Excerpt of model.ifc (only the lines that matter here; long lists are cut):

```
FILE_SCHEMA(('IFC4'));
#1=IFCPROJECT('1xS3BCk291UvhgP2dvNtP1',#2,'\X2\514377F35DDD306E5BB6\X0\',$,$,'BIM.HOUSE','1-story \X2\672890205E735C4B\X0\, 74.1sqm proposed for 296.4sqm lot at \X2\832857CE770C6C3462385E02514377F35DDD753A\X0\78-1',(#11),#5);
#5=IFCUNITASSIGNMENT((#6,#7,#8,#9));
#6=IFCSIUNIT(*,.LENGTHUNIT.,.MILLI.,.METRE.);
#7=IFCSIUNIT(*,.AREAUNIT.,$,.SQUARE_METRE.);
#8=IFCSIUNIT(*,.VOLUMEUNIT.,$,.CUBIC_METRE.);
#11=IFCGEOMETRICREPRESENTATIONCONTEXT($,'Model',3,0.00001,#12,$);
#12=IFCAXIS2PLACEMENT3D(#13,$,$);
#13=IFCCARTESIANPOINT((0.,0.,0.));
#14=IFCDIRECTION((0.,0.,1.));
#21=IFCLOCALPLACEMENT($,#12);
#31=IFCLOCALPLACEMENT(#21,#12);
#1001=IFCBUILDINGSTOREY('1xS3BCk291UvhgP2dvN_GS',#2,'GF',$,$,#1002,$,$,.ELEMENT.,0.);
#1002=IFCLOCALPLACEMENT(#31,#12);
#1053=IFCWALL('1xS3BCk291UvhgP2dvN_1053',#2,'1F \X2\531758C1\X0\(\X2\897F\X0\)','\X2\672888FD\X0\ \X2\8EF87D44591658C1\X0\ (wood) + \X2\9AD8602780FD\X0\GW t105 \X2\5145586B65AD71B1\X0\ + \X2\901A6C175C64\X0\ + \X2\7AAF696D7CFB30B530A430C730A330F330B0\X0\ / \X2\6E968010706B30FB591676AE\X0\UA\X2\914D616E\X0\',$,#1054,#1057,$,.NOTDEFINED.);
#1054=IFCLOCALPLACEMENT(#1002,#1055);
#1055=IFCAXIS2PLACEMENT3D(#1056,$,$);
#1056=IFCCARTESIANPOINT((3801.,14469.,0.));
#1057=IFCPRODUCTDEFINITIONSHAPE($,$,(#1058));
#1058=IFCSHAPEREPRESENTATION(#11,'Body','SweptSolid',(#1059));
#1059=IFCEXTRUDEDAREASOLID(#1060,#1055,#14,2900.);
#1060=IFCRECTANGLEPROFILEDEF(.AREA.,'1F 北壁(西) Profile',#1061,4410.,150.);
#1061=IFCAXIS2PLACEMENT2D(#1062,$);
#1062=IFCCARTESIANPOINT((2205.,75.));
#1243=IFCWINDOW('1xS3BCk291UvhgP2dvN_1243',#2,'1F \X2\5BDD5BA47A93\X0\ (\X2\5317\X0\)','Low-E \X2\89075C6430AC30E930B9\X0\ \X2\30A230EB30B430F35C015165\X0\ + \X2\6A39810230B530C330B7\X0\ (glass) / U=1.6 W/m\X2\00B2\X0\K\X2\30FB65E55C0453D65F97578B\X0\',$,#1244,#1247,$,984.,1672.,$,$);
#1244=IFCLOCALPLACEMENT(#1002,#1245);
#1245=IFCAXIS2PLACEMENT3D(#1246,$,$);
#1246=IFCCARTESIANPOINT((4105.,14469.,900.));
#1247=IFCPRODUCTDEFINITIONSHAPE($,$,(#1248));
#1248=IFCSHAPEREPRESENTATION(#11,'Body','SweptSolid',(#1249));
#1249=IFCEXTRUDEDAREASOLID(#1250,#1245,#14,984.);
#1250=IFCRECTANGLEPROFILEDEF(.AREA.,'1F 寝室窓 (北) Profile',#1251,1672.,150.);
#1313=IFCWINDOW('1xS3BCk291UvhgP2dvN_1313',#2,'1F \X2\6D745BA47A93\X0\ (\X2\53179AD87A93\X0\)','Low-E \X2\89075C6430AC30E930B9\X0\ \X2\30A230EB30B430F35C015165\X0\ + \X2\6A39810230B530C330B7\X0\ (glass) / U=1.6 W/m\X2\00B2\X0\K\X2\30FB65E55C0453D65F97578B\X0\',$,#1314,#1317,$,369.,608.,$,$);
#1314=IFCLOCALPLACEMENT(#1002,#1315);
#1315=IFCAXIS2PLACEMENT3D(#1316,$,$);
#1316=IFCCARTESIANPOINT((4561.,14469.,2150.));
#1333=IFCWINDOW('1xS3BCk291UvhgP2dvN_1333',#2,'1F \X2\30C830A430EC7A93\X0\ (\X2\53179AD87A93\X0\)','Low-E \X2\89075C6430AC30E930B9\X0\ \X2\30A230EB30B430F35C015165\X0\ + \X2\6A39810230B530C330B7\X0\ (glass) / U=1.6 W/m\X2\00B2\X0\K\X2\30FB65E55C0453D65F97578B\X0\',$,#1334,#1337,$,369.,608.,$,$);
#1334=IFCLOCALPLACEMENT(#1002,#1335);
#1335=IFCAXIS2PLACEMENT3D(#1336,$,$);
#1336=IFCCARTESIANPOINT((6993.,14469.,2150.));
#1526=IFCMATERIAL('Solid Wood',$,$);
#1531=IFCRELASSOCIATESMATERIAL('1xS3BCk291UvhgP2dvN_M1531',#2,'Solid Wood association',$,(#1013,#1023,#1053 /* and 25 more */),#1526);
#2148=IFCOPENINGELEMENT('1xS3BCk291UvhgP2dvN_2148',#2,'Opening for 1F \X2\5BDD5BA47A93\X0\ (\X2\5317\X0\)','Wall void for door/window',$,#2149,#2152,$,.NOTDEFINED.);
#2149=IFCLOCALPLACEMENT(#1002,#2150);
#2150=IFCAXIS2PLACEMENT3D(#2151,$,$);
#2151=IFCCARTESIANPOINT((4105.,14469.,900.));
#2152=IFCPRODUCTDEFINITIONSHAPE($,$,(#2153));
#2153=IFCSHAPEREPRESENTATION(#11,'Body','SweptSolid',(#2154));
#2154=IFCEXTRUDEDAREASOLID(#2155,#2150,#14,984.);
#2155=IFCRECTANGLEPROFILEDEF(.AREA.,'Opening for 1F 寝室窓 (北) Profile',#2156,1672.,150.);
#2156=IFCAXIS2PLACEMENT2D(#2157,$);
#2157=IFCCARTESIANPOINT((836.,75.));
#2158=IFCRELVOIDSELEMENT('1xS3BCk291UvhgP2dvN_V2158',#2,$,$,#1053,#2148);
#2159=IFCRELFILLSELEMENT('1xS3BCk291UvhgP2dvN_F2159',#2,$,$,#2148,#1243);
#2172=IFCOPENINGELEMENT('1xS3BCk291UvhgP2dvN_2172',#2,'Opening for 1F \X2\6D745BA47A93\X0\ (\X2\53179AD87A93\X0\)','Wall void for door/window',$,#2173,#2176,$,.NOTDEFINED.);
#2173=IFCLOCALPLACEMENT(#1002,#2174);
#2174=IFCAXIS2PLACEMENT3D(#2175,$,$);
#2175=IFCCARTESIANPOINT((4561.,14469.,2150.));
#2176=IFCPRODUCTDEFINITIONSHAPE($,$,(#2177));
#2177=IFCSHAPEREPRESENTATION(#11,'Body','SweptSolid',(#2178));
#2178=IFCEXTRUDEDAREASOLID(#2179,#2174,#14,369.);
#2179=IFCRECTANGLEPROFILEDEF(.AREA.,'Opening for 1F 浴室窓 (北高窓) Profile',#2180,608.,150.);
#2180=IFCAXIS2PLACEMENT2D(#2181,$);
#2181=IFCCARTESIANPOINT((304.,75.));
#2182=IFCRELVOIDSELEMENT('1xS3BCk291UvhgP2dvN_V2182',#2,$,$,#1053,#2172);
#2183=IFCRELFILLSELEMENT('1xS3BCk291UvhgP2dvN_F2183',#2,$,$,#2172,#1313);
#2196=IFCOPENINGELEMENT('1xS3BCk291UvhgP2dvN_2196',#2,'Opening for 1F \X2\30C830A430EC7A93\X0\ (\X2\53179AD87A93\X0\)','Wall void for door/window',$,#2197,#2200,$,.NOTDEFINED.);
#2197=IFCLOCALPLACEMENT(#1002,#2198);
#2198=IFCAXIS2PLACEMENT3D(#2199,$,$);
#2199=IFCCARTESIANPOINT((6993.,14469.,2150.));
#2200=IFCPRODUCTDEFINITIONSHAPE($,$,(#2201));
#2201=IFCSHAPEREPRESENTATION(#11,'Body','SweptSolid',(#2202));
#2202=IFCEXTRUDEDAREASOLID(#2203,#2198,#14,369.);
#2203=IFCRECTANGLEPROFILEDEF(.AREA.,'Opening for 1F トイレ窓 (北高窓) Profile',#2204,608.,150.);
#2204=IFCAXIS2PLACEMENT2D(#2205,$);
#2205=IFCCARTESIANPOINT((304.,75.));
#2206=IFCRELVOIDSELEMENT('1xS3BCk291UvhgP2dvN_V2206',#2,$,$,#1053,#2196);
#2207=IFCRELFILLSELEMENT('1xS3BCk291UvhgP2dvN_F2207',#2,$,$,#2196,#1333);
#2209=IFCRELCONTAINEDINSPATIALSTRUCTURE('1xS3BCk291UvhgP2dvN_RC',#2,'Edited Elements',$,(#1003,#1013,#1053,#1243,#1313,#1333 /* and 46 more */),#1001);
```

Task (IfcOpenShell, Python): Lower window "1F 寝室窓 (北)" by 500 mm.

```python
import numpy as np
import ifcopenshell
import ifcopenshell.api.geometry
import ifcopenshell.util.placement
import ifcopenshell.util.unit

model = ifcopenshell.open("model.ifc")
unit_scale = ifcopenshell.util.unit.calculate_unit_scale(model)

window = model.by_guid("1xS3BCk291UvhgP2dvN_1243")
opening = window.FillsVoids[0].RelatingOpeningElement
dz = -0.5 / unit_scale

shift = np.array([0.0, 0.0, dz])
# The window is not placed relative to its opening, so move both.
for product in (opening, window):
    matrix = ifcopenshell.util.placement.get_local_placement(product.ObjectPlacement)
    matrix[:3, 3] += shift
    ifcopenshell.api.geometry.edit_object_placement(model, product=product, matrix=matrix, is_si=False)

print(f"moved by {dz * unit_scale:+.3f} m")

model.write("model_v2.ifc")
```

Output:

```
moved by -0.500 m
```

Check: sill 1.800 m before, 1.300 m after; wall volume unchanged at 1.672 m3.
